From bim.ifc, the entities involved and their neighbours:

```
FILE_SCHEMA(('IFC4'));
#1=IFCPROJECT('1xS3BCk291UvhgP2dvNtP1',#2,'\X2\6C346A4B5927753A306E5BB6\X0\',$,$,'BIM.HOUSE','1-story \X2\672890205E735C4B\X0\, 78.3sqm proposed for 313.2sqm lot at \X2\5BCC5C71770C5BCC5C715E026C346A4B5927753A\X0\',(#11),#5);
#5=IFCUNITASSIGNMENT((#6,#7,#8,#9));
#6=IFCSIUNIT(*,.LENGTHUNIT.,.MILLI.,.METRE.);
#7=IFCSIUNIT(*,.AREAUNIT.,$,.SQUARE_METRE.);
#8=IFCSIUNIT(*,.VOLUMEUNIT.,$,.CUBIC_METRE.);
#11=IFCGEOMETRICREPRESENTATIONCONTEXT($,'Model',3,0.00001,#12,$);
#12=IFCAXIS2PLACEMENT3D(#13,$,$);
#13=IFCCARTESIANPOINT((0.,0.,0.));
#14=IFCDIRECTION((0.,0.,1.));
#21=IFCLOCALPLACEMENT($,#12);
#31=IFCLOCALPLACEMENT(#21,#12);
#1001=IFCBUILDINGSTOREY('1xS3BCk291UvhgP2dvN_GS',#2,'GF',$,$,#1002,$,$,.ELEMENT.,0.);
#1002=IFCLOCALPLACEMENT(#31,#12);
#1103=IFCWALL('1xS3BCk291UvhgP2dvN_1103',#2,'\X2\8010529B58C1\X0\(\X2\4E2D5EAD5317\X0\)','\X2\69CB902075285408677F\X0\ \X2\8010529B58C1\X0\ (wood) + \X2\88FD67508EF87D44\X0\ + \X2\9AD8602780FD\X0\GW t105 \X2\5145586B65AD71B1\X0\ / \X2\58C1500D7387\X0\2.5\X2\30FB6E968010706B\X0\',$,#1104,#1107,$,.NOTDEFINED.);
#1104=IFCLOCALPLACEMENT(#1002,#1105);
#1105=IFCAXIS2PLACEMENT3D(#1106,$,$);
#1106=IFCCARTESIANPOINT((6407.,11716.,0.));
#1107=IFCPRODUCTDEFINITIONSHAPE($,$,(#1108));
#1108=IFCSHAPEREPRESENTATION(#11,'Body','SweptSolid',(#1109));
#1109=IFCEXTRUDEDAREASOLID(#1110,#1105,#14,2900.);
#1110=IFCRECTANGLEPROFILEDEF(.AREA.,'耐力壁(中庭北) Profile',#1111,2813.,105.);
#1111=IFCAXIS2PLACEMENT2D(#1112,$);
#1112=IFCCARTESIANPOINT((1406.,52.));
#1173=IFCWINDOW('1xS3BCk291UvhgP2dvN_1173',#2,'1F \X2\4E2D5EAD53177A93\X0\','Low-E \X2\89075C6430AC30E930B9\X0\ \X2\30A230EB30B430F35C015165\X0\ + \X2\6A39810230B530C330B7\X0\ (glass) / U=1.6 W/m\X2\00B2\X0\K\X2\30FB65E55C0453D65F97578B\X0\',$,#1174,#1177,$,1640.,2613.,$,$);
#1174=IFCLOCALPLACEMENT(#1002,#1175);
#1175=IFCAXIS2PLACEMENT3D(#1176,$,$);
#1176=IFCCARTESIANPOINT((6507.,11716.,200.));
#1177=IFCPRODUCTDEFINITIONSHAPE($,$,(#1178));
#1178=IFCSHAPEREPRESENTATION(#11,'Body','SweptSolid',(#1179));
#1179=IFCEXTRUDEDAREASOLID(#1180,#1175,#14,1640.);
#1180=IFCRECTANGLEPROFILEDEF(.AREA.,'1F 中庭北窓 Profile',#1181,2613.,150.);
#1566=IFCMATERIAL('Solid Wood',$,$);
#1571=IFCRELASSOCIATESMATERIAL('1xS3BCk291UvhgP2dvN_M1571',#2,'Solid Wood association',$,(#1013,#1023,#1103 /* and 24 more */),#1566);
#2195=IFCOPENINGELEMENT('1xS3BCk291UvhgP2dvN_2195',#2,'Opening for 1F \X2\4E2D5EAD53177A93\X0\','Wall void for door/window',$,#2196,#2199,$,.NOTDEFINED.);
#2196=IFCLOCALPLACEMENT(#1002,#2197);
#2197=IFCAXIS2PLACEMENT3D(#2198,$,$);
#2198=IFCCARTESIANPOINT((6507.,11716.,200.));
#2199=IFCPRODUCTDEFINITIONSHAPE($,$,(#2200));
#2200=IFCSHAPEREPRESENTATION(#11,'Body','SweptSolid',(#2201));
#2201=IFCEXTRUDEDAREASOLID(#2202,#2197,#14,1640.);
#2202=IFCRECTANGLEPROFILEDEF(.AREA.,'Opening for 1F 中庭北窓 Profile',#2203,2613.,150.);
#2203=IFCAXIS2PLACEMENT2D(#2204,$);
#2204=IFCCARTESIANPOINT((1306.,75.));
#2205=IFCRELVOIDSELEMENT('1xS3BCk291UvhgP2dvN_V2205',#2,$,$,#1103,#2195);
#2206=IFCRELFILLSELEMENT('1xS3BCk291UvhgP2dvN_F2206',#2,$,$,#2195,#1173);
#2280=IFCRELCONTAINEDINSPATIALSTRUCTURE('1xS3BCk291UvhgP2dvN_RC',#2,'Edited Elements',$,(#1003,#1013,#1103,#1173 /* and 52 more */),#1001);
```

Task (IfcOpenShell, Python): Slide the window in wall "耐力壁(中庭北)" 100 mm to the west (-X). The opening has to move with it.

```python
import ifcopenshell
import ifcopenshell.api.geometry
import ifcopenshell.util.placement
import ifcopenshell.util.unit

model = ifcopenshell.open("bim.ifc")
unit_scale = ifcopenshell.util.unit.calculate_unit_scale(model)

window = model.by_id(1173)
opening = window.FillsVoids[0].RelatingOpeningElement
wall = opening.VoidsElements[0].RelatingBuildingElement

wall_matrix = ifcopenshell.util.placement.get_local_placement(wall.ObjectPlacement)
shift = wall_matrix[:3, 0] * -0.1 / unit_scale
before = ifcopenshell.util.placement.get_local_placement(window.ObjectPlacement)[:3, 3].copy()

# The window is not placed relative to its opening, so move both.
for product in (opening, window):
    matrix = ifcopenshell.util.placement.get_local_placement(product.ObjectPlacement)
    matrix[:3, 3] += shift
    ifcopenshell.api.geometry.edit_object_placement(model, product=product, matrix=matrix, is_si=False)

after = ifcopenshell.util.placement.get_local_placement(window.ObjectPlacement)[:3, 3]
print("window moved by", (after - before).round(3) + 0.0)

model.write("bim_v2.ifc")
```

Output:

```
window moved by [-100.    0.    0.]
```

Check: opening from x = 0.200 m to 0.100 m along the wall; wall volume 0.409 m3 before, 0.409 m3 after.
